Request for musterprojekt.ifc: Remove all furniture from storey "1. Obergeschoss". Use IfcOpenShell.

First a look at what the model holds.

```python
import ifcopenshell
import ifcopenshell.util.element

model = ifcopenshell.open("musterprojekt.ifc")
print(model.schema)
storey = next(s for s in model.by_type("IfcBuildingStorey") if s.Name == "1. Obergeschoss")
furniture = [e for e in ifcopenshell.util.element.get_decomposition(storey) if e.is_a("IfcFurnishingElement")]
seen = {}
for e in furniture:
    element_type = ifcopenshell.util.element.get_type(e)
    name = element_type.Name if element_type not in (None, e) else None
    seen[name] = seen.get(name, 0) + 1
for name, count in sorted(seen.items(), key=str):
    print(count, "x", name)
```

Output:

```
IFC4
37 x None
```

```python
import ifcopenshell
import ifcopenshell.api.root
import ifcopenshell.util.element

model = ifcopenshell.open("musterprojekt.ifc")

storey = next(s for s in model.by_type("IfcBuildingStorey") if s.Name == "1. Obergeschoss")
furniture = [e for e in ifcopenshell.util.element.get_decomposition(storey) if e.is_a("IfcFurnishingElement")]

for e in furniture:
    ifcopenshell.api.root.remove_product(model, product=e)
print(len(furniture), "removed")

model.write("musterprojekt-out.ifc")
```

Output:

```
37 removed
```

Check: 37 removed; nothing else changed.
